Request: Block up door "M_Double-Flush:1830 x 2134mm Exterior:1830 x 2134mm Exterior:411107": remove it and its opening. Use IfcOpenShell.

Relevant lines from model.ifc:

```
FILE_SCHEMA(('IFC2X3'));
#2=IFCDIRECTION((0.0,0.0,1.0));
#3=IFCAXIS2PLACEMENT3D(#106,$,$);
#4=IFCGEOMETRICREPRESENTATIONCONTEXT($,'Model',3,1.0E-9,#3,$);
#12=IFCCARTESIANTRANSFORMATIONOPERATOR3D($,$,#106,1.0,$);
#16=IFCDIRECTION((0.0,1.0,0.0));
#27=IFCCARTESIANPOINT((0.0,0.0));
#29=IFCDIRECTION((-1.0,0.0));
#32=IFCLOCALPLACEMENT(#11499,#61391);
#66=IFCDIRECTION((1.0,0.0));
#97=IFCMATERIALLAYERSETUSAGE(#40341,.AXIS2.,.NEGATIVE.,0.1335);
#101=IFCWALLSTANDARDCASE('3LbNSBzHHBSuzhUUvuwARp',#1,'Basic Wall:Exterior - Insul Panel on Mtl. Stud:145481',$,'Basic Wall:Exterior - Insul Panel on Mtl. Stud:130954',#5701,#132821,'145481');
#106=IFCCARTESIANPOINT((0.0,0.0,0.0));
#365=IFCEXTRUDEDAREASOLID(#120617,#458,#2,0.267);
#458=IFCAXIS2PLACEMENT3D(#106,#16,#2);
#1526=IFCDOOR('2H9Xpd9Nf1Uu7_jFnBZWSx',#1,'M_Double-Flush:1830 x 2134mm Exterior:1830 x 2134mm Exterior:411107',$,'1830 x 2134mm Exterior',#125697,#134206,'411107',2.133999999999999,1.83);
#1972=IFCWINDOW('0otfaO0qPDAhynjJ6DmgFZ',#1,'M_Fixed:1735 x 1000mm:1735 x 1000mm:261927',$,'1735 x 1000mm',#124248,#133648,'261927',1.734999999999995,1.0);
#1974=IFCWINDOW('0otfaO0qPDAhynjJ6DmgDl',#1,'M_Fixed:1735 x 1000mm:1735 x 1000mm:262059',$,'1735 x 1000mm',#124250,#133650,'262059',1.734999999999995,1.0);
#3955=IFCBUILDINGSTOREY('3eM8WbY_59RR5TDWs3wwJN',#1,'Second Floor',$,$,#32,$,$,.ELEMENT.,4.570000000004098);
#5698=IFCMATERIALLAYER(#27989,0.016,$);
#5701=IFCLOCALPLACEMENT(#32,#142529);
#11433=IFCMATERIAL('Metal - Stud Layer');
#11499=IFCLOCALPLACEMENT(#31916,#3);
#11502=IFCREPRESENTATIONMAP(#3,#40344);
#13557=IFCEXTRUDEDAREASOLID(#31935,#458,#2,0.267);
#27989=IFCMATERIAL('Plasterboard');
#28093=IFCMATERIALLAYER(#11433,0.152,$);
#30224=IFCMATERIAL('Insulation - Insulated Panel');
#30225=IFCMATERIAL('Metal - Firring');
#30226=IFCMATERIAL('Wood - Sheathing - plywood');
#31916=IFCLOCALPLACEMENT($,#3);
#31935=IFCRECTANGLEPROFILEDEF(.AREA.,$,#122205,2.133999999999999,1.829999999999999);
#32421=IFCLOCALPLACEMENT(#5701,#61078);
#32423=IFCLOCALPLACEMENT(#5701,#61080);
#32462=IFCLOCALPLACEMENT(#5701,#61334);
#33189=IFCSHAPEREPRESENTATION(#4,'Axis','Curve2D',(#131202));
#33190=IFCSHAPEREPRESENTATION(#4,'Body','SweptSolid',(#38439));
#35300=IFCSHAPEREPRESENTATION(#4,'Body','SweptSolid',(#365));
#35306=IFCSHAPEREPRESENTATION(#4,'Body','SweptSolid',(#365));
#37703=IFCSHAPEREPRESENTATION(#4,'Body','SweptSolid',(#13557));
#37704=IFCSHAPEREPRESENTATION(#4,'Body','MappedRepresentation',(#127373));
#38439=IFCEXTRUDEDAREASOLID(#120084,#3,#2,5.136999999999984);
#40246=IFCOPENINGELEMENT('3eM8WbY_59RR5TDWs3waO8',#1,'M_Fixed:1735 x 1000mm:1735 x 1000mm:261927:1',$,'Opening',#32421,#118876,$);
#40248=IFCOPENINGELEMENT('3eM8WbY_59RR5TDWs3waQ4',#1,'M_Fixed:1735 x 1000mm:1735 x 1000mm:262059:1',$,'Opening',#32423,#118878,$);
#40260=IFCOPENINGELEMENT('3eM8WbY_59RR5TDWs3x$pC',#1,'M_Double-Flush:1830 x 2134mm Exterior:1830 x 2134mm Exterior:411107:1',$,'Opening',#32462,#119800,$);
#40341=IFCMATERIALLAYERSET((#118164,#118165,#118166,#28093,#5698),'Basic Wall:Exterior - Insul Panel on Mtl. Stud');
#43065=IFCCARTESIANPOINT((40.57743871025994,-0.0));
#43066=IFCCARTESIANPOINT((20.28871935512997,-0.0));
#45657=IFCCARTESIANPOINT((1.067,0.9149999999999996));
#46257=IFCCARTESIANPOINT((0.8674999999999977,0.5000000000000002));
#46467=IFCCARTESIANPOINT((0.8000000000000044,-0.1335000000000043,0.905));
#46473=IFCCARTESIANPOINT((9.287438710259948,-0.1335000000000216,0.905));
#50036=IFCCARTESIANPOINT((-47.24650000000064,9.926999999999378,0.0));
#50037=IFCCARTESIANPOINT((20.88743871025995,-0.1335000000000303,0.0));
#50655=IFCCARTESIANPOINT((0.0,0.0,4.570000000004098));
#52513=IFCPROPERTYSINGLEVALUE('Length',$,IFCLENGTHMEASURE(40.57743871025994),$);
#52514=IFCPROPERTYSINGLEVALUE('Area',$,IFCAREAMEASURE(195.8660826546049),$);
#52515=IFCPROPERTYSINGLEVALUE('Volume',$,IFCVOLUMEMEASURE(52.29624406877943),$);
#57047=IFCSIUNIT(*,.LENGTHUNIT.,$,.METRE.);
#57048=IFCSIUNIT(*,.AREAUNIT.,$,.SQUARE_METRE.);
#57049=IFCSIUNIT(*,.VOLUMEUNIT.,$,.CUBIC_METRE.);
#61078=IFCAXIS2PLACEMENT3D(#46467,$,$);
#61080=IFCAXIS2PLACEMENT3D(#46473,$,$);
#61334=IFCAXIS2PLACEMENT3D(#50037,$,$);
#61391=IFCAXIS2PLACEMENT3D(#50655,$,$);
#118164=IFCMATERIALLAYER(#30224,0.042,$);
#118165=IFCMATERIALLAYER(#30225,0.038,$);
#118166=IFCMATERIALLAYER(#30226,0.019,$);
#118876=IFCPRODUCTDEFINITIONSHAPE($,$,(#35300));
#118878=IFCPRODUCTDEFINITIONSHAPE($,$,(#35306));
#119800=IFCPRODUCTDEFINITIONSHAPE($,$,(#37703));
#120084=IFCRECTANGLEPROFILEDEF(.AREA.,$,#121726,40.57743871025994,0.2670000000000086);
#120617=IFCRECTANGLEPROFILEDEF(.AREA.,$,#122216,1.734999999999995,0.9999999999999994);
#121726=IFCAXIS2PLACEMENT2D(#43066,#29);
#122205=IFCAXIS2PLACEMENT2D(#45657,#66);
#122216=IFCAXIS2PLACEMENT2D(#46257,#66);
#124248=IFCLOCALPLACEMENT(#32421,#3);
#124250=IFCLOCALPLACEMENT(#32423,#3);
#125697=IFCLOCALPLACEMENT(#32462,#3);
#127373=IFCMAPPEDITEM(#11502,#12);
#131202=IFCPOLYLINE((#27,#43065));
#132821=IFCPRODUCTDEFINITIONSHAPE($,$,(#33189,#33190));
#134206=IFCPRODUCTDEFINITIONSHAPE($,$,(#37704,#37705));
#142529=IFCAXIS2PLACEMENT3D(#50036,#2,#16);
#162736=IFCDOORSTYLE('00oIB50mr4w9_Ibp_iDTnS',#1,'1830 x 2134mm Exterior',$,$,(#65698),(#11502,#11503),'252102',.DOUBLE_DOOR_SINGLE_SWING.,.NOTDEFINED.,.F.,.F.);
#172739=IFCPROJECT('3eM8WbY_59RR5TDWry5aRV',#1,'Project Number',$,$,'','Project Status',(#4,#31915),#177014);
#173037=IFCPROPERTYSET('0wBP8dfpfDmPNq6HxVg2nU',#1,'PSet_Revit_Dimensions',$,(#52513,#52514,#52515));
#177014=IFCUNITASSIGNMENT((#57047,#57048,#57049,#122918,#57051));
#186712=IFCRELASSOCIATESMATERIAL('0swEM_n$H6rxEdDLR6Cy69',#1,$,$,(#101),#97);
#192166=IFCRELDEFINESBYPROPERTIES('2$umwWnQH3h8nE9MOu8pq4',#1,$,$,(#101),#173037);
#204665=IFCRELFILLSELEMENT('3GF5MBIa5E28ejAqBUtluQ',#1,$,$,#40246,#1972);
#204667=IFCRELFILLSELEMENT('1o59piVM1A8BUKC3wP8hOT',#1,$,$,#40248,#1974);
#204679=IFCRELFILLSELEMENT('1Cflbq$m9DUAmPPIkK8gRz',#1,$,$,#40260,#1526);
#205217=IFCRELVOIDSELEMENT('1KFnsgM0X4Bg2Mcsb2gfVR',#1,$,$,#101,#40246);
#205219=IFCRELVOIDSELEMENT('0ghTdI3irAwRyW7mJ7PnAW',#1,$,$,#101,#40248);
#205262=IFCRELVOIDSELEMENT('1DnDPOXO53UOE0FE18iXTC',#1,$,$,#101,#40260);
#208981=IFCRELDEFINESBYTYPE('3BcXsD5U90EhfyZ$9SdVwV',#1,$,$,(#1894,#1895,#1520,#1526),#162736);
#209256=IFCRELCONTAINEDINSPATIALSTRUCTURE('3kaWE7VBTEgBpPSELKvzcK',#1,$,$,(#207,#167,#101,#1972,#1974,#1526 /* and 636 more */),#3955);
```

```python
import ifcopenshell
import ifcopenshell.api.feature
import ifcopenshell.api.pset
import ifcopenshell.api.root
import ifcopenshell.geom
import ifcopenshell.util.element
import ifcopenshell.util.shape
import ifcopenshell.util.unit

model = ifcopenshell.open("model.ifc")
area_scale = ifcopenshell.util.unit.calculate_unit_scale(model, "AREAUNIT")
volume_scale = ifcopenshell.util.unit.calculate_unit_scale(model, "VOLUMEUNIT")
settings = ifcopenshell.geom.settings()


def volume(element):
    """Net volume in cubic metres, openings subtracted."""
    shape = ifcopenshell.geom.create_shape(settings, element)
    return ifcopenshell.util.shape.get_volume(shape.geometry)


door = model.by_guid("2H9Xpd9Nf1Uu7_jFnBZWSx")
opening = door.FillsVoids[0].RelatingOpeningElement
wall = opening.VoidsElements[0].RelatingBuildingElement
before = volume(wall)

ifcopenshell.api.root.remove_product(model, product=door)
ifcopenshell.api.feature.remove_feature(model, feature=opening)

after = volume(wall)
thickness = 0.267  # wall thickness in metres

# Update the wall's stored quantities.
pset = model.by_id(ifcopenshell.util.element.get_pset(wall, "PSet_Revit_Dimensions", should_inherit=False)["id"])
ifcopenshell.api.pset.edit_pset(model, pset=pset, properties={
    "Area": model.create_entity("IfcAreaMeasure", after / thickness / area_scale),
    "Volume": model.create_entity("IfcVolumeMeasure", after / volume_scale),
})

print(f"wall volume {before:.3f} -> {after:.3f} m3")

model.write("model-out.ifc")
```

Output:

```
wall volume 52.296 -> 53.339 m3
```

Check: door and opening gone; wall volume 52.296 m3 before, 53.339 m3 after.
